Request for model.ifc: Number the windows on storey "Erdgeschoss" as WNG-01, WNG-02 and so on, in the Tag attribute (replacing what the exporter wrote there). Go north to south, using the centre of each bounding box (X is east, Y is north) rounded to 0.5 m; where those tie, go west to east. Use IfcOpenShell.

First a look at what the model holds.

```python
import ifcopenshell
import ifcopenshell.util.element
import ifcopenshell.util.placement

model = ifcopenshell.open("model.ifc")
print(model.schema)
storey = next(s for s in model.by_type("IfcBuildingStorey") if s.Name == "Erdgeschoss")
windows = [e for e in ifcopenshell.util.element.get_decomposition(storey) if e.is_a("IfcWindow")]
for e in sorted(windows, key=lambda e: e.id()):
    origin = ifcopenshell.util.placement.get_local_placement(e.ObjectPlacement)[:3, 3]
    print(e.id(), e.Tag, e.Name, origin.round(2) + 0.0, sep=" | ")
```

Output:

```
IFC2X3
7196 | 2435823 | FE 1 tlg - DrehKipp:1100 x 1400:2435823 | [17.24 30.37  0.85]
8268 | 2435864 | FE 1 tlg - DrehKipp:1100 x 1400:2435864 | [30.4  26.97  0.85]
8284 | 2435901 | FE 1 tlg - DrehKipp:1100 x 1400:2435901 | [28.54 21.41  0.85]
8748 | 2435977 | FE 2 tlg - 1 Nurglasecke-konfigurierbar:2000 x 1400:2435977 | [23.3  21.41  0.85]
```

```python
import ifcopenshell
import ifcopenshell.geom
import ifcopenshell.util.element
import ifcopenshell.util.shape

model = ifcopenshell.open("model.ifc")
settings = ifcopenshell.geom.settings()
settings.set("use-world-coords", True)


def centre(element):
    shape = ifcopenshell.geom.create_shape(settings, element)
    return ifcopenshell.util.shape.get_bbox_centroid(shape.geometry)


storey = next(s for s in model.by_type("IfcBuildingStorey") if s.Name == "Erdgeschoss")
windows = [e for e in ifcopenshell.util.element.get_decomposition(storey) if e.is_a("IfcWindow")]

# Insertion points can sit at a corner or the storey origin, so sort by the geometry (in metres).
centres = {e: centre(e) for e in windows}
windows.sort(key=lambda e: (-round(centres[e][1] / 0.5), centres[e][0]))

for i, e in enumerate(windows, start=1):
    number = f"WNG-{i:02d}"
    e.Tag = number
    print(e.id(), number)

model.write("model_updated.ifc")
```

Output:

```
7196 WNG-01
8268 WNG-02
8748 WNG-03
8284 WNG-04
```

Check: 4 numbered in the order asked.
